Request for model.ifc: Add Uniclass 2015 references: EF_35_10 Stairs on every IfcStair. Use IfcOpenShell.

First a look at what the model holds.

```python
import ifcopenshell

model = ifcopenshell.open("model.ifc")
print(model.schema)
print("classifications:", [c.Name for c in model.by_type("IfcClassification")])
for ifc_class in ("IfcDoor", "IfcRoof", "IfcStair", "IfcWall", "IfcWindow"):
    print(ifc_class, len(model.by_type(ifc_class)))
```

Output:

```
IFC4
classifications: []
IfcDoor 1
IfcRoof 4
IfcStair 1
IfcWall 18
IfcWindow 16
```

```python
import ifcopenshell
import ifcopenshell.api.classification

model = ifcopenshell.open("model.ifc")

system = ifcopenshell.api.classification.add_classification(model, classification="Uniclass 2015")

codes = {
    "IfcStair": ("EF_35_10", "Stairs"),
}
for ifc_class, (code, name) in codes.items():
    products = model.by_type(ifc_class)
    ifcopenshell.api.classification.add_reference(
        model, products=products, classification=system, identification=code, name=name
    )
    print(code, len(products))

model.write("model-out.ifc")
```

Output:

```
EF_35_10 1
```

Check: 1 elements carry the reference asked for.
